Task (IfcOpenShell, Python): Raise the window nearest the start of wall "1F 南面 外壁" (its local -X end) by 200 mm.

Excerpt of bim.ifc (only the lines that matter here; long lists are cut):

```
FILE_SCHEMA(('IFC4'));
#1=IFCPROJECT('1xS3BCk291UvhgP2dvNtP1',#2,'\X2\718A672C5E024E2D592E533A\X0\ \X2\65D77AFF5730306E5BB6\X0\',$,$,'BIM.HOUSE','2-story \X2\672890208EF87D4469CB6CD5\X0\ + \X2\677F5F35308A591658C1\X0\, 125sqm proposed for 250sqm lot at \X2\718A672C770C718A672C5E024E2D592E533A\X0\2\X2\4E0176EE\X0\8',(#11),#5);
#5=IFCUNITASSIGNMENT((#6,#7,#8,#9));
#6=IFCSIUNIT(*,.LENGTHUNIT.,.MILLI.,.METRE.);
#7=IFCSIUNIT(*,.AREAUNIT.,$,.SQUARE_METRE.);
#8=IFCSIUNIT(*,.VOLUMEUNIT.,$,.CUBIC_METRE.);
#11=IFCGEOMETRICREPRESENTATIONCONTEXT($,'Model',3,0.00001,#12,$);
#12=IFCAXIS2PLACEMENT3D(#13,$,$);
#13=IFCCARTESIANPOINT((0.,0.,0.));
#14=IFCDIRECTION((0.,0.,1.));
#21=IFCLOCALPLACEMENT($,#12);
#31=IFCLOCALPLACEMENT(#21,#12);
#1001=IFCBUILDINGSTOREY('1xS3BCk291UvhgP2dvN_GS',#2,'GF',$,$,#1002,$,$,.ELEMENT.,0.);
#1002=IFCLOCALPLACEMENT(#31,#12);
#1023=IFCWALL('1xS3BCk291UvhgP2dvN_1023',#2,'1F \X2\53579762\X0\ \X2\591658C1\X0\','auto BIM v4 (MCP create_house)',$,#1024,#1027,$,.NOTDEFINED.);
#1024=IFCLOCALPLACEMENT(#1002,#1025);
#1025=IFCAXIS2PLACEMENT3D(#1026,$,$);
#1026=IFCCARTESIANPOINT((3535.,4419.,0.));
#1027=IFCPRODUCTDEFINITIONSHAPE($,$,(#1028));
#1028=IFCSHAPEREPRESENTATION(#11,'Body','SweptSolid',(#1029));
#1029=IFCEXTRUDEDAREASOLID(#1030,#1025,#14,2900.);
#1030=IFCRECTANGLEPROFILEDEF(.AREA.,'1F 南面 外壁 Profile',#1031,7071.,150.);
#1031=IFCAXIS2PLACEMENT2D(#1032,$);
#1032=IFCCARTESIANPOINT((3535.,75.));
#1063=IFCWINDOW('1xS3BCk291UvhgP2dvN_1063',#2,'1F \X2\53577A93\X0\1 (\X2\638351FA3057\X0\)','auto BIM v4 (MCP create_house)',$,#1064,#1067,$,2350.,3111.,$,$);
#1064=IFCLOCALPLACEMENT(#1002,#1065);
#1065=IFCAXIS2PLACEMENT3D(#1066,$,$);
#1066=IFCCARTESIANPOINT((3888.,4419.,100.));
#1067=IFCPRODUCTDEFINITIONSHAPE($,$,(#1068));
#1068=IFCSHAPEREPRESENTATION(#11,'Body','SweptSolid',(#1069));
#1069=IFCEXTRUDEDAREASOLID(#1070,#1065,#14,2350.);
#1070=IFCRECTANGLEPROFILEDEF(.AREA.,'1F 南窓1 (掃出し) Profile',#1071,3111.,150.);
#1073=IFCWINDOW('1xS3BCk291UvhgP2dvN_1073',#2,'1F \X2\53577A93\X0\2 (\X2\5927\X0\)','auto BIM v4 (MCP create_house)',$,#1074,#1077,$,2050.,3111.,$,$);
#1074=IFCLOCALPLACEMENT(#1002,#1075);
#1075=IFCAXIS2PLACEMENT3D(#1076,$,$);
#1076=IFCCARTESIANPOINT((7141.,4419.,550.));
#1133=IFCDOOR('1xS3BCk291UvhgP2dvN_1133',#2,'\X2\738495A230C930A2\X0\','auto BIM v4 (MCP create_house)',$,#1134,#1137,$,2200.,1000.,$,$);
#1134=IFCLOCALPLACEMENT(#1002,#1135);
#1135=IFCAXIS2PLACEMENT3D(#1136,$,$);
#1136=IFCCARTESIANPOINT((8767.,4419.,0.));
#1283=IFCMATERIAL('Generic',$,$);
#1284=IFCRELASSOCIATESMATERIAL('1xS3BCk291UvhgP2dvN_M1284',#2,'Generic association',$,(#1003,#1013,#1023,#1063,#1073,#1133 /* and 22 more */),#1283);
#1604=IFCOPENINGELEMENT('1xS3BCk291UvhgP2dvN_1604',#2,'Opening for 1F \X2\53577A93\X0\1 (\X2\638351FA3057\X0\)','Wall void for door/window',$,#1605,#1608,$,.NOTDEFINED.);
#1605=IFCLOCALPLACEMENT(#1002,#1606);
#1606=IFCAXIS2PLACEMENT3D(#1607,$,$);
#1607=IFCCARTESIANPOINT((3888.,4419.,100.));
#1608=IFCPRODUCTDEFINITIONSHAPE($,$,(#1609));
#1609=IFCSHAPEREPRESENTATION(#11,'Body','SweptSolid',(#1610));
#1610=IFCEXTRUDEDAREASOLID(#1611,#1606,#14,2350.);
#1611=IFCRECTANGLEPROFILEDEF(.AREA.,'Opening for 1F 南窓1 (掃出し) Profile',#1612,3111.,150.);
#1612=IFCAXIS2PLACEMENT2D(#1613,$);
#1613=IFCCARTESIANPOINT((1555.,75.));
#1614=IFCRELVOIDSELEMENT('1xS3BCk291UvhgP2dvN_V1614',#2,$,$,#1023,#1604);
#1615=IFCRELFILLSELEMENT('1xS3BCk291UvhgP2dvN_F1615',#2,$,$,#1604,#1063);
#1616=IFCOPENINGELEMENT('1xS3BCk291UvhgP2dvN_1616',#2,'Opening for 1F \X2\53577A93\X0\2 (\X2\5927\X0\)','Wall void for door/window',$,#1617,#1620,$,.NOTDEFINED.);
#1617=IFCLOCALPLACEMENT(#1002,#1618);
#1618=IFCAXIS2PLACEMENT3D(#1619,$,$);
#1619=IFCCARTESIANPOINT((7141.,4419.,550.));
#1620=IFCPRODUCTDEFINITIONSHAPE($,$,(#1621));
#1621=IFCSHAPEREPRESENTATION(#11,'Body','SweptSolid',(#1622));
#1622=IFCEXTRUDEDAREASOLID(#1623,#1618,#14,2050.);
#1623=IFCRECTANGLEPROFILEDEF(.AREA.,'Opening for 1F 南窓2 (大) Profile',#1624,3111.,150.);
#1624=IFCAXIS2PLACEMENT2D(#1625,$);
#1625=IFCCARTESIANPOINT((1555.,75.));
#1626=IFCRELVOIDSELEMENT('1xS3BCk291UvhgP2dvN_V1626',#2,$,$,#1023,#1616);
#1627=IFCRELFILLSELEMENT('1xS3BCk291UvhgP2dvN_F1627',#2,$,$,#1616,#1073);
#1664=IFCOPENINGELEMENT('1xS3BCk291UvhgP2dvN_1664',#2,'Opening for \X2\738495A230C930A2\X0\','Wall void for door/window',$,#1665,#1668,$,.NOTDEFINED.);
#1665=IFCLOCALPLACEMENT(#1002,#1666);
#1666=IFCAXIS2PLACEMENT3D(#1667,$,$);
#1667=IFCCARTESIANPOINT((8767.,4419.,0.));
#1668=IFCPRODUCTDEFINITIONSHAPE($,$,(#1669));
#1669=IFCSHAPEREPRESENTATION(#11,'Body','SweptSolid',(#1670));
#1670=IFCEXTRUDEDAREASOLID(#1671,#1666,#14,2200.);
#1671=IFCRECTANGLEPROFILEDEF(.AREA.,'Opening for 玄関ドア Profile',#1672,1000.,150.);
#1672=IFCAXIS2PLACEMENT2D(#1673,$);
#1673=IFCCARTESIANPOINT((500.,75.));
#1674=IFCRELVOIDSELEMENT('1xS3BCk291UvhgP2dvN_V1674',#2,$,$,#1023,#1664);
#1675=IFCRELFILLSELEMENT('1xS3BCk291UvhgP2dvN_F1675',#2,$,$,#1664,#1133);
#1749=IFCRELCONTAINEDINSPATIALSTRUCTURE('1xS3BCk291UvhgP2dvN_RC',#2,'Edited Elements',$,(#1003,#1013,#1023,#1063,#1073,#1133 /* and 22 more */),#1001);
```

```python
import numpy as np
import ifcopenshell
import ifcopenshell.api.geometry
import ifcopenshell.util.placement
import ifcopenshell.util.unit

model = ifcopenshell.open("bim.ifc")
unit_scale = ifcopenshell.util.unit.calculate_unit_scale(model)

window = model.by_id(1063)
opening = window.FillsVoids[0].RelatingOpeningElement
dz = 0.2 / unit_scale

shift = np.array([0.0, 0.0, dz])
# The window is not placed relative to its opening, so move both.
for product in (opening, window):
    matrix = ifcopenshell.util.placement.get_local_placement(product.ObjectPlacement)
    matrix[:3, 3] += shift
    ifcopenshell.api.geometry.edit_object_placement(model, product=product, matrix=matrix, is_si=False)

print(f"moved by {dz * unit_scale:+.3f} m")

model.write("bim-out.ifc")
```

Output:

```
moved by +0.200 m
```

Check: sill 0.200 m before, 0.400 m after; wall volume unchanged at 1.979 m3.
